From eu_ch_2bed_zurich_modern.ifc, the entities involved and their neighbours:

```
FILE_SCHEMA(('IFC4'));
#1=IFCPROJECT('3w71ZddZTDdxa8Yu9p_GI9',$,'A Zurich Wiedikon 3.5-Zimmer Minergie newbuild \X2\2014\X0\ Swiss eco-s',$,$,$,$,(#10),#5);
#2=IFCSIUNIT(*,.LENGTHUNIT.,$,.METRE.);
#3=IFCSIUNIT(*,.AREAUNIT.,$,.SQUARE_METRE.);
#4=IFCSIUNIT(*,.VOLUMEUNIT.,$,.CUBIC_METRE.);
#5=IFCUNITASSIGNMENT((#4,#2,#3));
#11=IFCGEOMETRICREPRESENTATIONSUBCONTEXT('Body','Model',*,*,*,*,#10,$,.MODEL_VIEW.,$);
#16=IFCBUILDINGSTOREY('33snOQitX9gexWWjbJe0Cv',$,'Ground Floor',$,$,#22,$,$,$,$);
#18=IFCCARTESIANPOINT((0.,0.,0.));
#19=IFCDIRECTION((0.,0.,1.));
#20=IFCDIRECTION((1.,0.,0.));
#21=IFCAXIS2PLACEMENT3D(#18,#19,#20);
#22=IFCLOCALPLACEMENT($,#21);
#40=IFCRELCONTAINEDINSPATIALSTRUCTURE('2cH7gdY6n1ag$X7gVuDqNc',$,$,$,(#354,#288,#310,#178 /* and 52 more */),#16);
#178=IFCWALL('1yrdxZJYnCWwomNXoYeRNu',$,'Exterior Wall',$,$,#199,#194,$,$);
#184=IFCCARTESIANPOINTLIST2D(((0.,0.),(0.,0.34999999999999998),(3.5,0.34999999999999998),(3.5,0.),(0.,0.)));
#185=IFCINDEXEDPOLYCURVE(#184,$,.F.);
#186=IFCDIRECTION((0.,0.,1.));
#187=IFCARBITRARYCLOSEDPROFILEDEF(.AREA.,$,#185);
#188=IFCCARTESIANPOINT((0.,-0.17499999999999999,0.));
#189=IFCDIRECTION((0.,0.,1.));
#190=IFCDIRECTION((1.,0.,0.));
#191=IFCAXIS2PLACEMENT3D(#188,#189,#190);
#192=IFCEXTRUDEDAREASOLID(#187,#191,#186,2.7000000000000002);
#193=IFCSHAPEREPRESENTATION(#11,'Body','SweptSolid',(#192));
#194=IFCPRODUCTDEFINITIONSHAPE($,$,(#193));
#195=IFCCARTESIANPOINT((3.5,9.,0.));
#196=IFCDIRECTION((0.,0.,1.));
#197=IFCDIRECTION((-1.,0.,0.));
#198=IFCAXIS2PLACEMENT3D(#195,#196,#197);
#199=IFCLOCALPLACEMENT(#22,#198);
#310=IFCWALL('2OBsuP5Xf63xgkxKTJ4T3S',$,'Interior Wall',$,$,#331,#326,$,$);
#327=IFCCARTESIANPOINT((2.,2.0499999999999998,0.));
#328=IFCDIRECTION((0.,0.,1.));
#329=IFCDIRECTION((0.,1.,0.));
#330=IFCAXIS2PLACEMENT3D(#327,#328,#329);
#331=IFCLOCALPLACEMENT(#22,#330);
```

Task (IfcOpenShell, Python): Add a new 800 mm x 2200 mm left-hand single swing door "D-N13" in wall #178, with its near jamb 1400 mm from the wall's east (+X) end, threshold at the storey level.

```python
import numpy as np
import ifcopenshell
import ifcopenshell.api.feature
import ifcopenshell.api.geometry
import ifcopenshell.api.root
import ifcopenshell.api.spatial
import ifcopenshell.geom
import ifcopenshell.util.element
import ifcopenshell.util.placement
import ifcopenshell.util.representation
import ifcopenshell.util.shape
import ifcopenshell.util.unit

model = ifcopenshell.open("eu_ch_2bed_zurich_modern.ifc")
unit_scale = ifcopenshell.util.unit.calculate_unit_scale(model)
settings = ifcopenshell.geom.settings()


def volume(element):
    """Net volume in cubic metres, openings subtracted."""
    shape = ifcopenshell.geom.create_shape(settings, element)
    return ifcopenshell.util.shape.get_volume(shape.geometry)


wall = model.by_guid("1yrdxZJYnCWwomNXoYeRNu")
storey = ifcopenshell.util.element.get_container(wall, ifc_class="IfcBuildingStorey")
context = ifcopenshell.util.representation.get_context(model, "Model", "Body", "MODEL_VIEW")
before = volume(wall)

width, height, from_end, sill = 0.8, 2.2, 1.4, 0.0  # metres

# The wall runs along its own X axis, and the end named is its -X end.
wall_shape = ifcopenshell.geom.create_shape(settings, wall)
x, y, z = ifcopenshell.util.shape.get_vertices(wall_shape.geometry).T
start = x.min() + from_end
face, thickness = float(y.min()), float(y.max() - y.min())
wall_matrix = ifcopenshell.util.placement.get_local_placement(wall.ObjectPlacement)
level = ifcopenshell.util.placement.get_local_placement(storey.ObjectPlacement)[2, 3]


def in_wall(x, y):
    """Placement at x, y metres in the wall's axes, at sill height."""
    matrix = wall_matrix.copy()
    matrix[:, 3] = wall_matrix @ np.array([x / unit_scale, y / unit_scale, 0.0, 1.0])
    matrix[2, 3] = level + sill / unit_scale
    return matrix


# Opening: a box that overshoots both wall faces by 50 mm.
opening = ifcopenshell.api.root.create_entity(model, ifc_class="IfcOpeningElement", predefined_type="OPENING")
box = ifcopenshell.api.geometry.add_wall_representation(
    model, context=context, length=width, height=height, thickness=thickness + 0.1
)
ifcopenshell.api.geometry.assign_representation(model, product=opening, representation=box)
ifcopenshell.api.geometry.edit_object_placement(model, product=opening, matrix=in_wall(start, face - 0.05), is_si=False)
ifcopenshell.api.feature.add_feature(model, feature=opening, element=wall)

door = ifcopenshell.api.root.create_entity(model, ifc_class="IfcDoor", name="D-N13", predefined_type="DOOR")
door.OverallWidth, door.OverallHeight = width / unit_scale, height / unit_scale
door.OperationType = "SINGLE_SWING_LEFT"
body = ifcopenshell.api.geometry.add_door_representation(
    model,
    context=context,
    overall_width=door.OverallWidth,
    overall_height=door.OverallHeight,
    operation_type="SINGLE_SWING_LEFT",
    lining_properties={"LiningDepth": thickness / unit_scale, "ThresholdDepth": thickness / unit_scale},
)
ifcopenshell.api.geometry.assign_representation(model, product=door, representation=body)
ifcopenshell.api.spatial.assign_container(model, products=[door], relating_structure=storey)
ifcopenshell.api.feature.add_filling(model, opening=opening, element=door)

# The lining spans the wall, so the door starts at the wall face.
ifcopenshell.api.geometry.edit_object_placement(model, product=door, matrix=in_wall(start, face), is_si=False)

after = volume(wall)

print(f"wall volume {before:.3f} -> {after:.3f} m3")

model.write("eu_ch_2bed_zurich_modern_updated.ifc")
```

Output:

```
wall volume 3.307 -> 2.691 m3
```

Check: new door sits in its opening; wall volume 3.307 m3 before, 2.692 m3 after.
